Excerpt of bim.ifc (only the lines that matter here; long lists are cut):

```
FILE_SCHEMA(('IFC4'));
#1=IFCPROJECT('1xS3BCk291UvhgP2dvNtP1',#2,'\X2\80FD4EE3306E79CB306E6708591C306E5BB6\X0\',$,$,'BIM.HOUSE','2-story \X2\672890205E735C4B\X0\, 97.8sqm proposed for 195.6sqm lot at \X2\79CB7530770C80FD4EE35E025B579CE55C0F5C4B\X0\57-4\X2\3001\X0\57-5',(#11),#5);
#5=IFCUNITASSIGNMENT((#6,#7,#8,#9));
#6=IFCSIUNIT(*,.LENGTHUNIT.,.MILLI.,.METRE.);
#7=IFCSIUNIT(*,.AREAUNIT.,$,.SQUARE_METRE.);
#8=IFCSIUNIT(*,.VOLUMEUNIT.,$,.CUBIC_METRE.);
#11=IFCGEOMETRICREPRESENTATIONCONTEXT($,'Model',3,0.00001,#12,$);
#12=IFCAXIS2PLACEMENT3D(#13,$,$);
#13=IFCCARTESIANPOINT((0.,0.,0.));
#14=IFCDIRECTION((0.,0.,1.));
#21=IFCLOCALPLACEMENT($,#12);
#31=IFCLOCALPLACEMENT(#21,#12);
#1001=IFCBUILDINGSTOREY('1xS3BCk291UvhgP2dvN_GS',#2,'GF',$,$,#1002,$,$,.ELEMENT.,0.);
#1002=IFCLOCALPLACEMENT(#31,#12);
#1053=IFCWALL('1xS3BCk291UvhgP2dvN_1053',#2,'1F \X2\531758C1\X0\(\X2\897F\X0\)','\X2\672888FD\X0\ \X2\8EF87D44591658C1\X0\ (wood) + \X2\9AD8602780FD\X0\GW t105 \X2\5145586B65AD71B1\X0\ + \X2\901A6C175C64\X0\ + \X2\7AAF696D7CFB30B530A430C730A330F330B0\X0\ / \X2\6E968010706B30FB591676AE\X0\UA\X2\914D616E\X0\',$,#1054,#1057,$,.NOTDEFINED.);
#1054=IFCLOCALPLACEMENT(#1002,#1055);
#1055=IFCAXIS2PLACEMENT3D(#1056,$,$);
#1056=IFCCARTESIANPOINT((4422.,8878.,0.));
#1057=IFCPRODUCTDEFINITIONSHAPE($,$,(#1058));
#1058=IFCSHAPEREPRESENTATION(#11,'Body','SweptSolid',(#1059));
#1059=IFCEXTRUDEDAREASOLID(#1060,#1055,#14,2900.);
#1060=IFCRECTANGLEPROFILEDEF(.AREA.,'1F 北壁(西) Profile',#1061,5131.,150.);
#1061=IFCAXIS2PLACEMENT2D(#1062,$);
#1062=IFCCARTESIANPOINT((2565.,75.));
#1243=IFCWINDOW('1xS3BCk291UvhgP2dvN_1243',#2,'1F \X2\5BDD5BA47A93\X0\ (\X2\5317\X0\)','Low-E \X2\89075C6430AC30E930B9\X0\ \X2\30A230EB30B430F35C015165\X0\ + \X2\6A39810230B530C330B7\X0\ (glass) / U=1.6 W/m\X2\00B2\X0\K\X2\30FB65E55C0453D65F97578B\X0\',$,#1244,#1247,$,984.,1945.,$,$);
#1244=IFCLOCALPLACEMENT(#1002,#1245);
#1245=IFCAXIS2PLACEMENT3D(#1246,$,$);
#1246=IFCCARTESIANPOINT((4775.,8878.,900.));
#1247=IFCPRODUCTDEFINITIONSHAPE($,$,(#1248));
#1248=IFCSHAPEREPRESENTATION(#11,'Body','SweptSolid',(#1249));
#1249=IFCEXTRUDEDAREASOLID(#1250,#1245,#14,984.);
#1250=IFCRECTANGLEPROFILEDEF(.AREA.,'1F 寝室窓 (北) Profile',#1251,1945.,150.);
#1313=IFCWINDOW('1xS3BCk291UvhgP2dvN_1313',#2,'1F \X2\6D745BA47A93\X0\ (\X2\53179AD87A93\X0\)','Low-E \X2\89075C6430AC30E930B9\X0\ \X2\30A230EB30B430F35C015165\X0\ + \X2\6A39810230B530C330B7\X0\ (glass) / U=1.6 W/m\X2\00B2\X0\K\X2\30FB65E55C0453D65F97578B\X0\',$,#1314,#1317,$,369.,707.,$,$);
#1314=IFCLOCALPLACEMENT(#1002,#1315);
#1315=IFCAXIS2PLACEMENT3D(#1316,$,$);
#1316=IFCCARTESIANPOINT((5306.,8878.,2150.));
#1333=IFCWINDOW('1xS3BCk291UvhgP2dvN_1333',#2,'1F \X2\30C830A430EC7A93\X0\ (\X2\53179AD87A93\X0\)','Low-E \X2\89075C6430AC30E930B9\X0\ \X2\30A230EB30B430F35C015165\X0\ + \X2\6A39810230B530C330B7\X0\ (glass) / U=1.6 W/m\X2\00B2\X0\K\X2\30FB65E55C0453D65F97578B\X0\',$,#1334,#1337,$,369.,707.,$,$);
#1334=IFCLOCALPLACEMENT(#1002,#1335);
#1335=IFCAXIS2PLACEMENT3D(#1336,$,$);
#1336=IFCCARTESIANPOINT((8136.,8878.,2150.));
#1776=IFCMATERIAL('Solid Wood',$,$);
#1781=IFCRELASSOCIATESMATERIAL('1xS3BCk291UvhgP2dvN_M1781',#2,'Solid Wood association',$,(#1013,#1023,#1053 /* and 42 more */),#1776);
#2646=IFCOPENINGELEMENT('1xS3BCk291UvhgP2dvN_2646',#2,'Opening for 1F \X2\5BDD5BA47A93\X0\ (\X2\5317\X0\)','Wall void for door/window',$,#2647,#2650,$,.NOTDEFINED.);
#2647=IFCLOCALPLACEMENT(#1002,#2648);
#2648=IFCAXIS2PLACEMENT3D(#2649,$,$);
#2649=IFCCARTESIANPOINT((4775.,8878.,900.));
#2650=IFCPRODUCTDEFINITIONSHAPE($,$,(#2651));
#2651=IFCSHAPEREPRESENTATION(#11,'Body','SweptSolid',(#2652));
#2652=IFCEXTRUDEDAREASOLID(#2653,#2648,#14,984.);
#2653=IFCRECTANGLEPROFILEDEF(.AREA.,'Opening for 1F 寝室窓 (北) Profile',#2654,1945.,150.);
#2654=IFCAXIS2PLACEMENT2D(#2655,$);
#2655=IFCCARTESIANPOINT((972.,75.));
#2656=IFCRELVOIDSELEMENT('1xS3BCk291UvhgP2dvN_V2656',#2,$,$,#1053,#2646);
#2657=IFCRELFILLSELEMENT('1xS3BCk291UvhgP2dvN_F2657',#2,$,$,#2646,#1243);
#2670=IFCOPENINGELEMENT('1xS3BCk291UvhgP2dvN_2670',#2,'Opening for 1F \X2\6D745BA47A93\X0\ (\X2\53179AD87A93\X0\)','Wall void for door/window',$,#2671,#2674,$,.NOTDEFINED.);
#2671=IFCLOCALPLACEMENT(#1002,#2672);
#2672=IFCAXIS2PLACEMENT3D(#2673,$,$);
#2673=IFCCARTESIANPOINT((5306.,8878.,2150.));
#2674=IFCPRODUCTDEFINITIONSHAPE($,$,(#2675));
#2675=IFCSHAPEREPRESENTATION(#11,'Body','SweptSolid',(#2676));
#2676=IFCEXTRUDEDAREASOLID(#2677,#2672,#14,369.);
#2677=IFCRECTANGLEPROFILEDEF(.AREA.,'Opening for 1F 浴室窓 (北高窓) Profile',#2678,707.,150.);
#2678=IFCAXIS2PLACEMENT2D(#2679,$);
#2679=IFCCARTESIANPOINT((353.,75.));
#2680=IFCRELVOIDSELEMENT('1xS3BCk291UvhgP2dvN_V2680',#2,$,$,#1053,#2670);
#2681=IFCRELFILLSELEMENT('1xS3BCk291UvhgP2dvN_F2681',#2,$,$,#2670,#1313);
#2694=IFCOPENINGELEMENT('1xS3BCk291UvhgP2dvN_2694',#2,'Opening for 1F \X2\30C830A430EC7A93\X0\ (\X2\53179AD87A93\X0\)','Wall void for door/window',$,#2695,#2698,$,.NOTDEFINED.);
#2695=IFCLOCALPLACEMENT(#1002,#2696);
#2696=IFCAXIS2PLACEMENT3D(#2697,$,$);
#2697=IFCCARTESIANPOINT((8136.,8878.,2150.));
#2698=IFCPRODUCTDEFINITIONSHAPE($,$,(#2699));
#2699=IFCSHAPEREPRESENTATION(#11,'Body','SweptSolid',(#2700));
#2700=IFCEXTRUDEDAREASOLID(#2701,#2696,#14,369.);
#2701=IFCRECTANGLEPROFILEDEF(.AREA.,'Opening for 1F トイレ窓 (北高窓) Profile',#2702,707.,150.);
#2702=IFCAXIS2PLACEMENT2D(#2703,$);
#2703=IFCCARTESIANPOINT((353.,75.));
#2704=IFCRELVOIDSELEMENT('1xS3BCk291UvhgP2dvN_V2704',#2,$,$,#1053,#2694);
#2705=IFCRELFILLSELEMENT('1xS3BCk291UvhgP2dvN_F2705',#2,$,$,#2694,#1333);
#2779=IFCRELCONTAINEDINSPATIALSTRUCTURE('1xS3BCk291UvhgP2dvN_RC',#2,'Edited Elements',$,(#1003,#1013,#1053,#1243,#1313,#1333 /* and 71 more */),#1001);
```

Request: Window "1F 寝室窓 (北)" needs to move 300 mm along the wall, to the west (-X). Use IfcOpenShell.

```python
import ifcopenshell
import ifcopenshell.api.geometry
import ifcopenshell.util.placement
import ifcopenshell.util.unit

model = ifcopenshell.open("bim.ifc")
unit_scale = ifcopenshell.util.unit.calculate_unit_scale(model)

window = model.by_guid("1xS3BCk291UvhgP2dvN_1243")
opening = window.FillsVoids[0].RelatingOpeningElement
wall = opening.VoidsElements[0].RelatingBuildingElement

wall_matrix = ifcopenshell.util.placement.get_local_placement(wall.ObjectPlacement)
shift = wall_matrix[:3, 0] * -0.3 / unit_scale
before = ifcopenshell.util.placement.get_local_placement(window.ObjectPlacement)[:3, 3].copy()

# The window is not placed relative to its opening, so move both.
for product in (opening, window):
    matrix = ifcopenshell.util.placement.get_local_placement(product.ObjectPlacement)
    matrix[:3, 3] += shift
    ifcopenshell.api.geometry.edit_object_placement(model, product=product, matrix=matrix, is_si=False)

after = ifcopenshell.util.placement.get_local_placement(window.ObjectPlacement)[:3, 3]
print("window moved by", (after - before).round(3) + 0.0)

model.write("bim_v2.ifc")
```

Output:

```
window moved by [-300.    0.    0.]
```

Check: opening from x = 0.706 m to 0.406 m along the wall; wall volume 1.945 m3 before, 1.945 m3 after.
